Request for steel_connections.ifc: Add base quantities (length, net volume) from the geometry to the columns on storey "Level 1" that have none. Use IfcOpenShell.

First a look at what the model holds.

```python
import ifcopenshell
import ifcopenshell.util.element
import ifcopenshell.util.unit

model = ifcopenshell.open("steel_connections.ifc")
print(model.schema)
for unit_type in ("LENGTHUNIT", "AREAUNIT", "VOLUMEUNIT"):
    print(unit_type, ifcopenshell.util.unit.calculate_unit_scale(model, unit_type))
storey = next(s for s in model.by_type("IfcBuildingStorey") if s.Name == "Level 1")
columns = [e for e in ifcopenshell.util.element.get_decomposition(storey) if e.is_a("IfcColumn")]
for e in sorted(columns, key=lambda e: e.id()):
    print(e.id(), e.is_a(), e.Name, list(ifcopenshell.util.element.get_psets(e, qtos_only=True)), sep=" | ")
```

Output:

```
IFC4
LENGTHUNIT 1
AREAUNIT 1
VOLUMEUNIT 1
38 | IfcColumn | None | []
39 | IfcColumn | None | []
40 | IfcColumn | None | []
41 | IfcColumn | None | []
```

```python
import ifcopenshell
import ifcopenshell.api.pset
import ifcopenshell.geom
import ifcopenshell.util.element
import ifcopenshell.util.shape
import ifcopenshell.util.unit

model = ifcopenshell.open("steel_connections.ifc")
unit_scale = ifcopenshell.util.unit.calculate_unit_scale(model)
volume_scale = ifcopenshell.util.unit.calculate_unit_scale(model, "VOLUMEUNIT")
settings = ifcopenshell.geom.settings()

storey = next(s for s in model.by_type("IfcBuildingStorey") if s.Name == "Level 1")
columns = [e for e in ifcopenshell.util.element.get_decomposition(storey) if e.is_a("IfcColumn")]

for e in sorted(columns, key=lambda e: e.id()):
    if ifcopenshell.util.element.get_psets(e, qtos_only=True, should_inherit=False):
        continue
    # Geometry comes back in metres, in the element's own axes.
    shape = ifcopenshell.geom.create_shape(settings, e)
    values = {
        "Length": ifcopenshell.util.shape.get_z(shape.geometry) / unit_scale,
        "NetVolume": ifcopenshell.util.shape.get_volume(shape.geometry) / volume_scale,
    }
    qto = ifcopenshell.api.pset.add_qto(model, product=e, name="Qto_ColumnBaseQuantities")
    ifcopenshell.api.pset.edit_qto(model, qto=qto, properties=values)
    print(e.id(), {k: round(v, 3) for k, v in values.items()})

model.write("steel_connections_edited.ifc")
```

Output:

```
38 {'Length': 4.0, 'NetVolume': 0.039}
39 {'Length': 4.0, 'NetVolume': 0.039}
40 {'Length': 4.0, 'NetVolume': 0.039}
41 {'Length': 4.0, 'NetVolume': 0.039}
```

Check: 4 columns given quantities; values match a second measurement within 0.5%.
